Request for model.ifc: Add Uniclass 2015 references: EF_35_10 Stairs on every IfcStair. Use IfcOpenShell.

First a look at what the model holds.

```python
import ifcopenshell

model = ifcopenshell.open("model.ifc")
print(model.schema)
print("classifications:", [c.Name for c in model.by_type("IfcClassification")])
for ifc_class in ("IfcDoor", "IfcRoof", "IfcStair", "IfcWall", "IfcWindow"):
    print(ifc_class, len(model.by_type(ifc_class)))
```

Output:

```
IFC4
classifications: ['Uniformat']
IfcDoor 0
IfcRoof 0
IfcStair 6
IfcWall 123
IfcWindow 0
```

```python
import ifcopenshell
import ifcopenshell.api.classification

model = ifcopenshell.open("model.ifc")

system = ifcopenshell.api.classification.add_classification(model, classification="Uniclass 2015")

codes = {
    "IfcStair": ("EF_35_10", "Stairs"),
}
for ifc_class, (code, name) in codes.items():
    products = model.by_type(ifc_class)
    ifcopenshell.api.classification.add_reference(
        model, products=products, classification=system, identification=code, name=name
    )
    print(code, len(products))

model.write("model_updated.ifc")
```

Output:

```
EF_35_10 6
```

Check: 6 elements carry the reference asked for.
